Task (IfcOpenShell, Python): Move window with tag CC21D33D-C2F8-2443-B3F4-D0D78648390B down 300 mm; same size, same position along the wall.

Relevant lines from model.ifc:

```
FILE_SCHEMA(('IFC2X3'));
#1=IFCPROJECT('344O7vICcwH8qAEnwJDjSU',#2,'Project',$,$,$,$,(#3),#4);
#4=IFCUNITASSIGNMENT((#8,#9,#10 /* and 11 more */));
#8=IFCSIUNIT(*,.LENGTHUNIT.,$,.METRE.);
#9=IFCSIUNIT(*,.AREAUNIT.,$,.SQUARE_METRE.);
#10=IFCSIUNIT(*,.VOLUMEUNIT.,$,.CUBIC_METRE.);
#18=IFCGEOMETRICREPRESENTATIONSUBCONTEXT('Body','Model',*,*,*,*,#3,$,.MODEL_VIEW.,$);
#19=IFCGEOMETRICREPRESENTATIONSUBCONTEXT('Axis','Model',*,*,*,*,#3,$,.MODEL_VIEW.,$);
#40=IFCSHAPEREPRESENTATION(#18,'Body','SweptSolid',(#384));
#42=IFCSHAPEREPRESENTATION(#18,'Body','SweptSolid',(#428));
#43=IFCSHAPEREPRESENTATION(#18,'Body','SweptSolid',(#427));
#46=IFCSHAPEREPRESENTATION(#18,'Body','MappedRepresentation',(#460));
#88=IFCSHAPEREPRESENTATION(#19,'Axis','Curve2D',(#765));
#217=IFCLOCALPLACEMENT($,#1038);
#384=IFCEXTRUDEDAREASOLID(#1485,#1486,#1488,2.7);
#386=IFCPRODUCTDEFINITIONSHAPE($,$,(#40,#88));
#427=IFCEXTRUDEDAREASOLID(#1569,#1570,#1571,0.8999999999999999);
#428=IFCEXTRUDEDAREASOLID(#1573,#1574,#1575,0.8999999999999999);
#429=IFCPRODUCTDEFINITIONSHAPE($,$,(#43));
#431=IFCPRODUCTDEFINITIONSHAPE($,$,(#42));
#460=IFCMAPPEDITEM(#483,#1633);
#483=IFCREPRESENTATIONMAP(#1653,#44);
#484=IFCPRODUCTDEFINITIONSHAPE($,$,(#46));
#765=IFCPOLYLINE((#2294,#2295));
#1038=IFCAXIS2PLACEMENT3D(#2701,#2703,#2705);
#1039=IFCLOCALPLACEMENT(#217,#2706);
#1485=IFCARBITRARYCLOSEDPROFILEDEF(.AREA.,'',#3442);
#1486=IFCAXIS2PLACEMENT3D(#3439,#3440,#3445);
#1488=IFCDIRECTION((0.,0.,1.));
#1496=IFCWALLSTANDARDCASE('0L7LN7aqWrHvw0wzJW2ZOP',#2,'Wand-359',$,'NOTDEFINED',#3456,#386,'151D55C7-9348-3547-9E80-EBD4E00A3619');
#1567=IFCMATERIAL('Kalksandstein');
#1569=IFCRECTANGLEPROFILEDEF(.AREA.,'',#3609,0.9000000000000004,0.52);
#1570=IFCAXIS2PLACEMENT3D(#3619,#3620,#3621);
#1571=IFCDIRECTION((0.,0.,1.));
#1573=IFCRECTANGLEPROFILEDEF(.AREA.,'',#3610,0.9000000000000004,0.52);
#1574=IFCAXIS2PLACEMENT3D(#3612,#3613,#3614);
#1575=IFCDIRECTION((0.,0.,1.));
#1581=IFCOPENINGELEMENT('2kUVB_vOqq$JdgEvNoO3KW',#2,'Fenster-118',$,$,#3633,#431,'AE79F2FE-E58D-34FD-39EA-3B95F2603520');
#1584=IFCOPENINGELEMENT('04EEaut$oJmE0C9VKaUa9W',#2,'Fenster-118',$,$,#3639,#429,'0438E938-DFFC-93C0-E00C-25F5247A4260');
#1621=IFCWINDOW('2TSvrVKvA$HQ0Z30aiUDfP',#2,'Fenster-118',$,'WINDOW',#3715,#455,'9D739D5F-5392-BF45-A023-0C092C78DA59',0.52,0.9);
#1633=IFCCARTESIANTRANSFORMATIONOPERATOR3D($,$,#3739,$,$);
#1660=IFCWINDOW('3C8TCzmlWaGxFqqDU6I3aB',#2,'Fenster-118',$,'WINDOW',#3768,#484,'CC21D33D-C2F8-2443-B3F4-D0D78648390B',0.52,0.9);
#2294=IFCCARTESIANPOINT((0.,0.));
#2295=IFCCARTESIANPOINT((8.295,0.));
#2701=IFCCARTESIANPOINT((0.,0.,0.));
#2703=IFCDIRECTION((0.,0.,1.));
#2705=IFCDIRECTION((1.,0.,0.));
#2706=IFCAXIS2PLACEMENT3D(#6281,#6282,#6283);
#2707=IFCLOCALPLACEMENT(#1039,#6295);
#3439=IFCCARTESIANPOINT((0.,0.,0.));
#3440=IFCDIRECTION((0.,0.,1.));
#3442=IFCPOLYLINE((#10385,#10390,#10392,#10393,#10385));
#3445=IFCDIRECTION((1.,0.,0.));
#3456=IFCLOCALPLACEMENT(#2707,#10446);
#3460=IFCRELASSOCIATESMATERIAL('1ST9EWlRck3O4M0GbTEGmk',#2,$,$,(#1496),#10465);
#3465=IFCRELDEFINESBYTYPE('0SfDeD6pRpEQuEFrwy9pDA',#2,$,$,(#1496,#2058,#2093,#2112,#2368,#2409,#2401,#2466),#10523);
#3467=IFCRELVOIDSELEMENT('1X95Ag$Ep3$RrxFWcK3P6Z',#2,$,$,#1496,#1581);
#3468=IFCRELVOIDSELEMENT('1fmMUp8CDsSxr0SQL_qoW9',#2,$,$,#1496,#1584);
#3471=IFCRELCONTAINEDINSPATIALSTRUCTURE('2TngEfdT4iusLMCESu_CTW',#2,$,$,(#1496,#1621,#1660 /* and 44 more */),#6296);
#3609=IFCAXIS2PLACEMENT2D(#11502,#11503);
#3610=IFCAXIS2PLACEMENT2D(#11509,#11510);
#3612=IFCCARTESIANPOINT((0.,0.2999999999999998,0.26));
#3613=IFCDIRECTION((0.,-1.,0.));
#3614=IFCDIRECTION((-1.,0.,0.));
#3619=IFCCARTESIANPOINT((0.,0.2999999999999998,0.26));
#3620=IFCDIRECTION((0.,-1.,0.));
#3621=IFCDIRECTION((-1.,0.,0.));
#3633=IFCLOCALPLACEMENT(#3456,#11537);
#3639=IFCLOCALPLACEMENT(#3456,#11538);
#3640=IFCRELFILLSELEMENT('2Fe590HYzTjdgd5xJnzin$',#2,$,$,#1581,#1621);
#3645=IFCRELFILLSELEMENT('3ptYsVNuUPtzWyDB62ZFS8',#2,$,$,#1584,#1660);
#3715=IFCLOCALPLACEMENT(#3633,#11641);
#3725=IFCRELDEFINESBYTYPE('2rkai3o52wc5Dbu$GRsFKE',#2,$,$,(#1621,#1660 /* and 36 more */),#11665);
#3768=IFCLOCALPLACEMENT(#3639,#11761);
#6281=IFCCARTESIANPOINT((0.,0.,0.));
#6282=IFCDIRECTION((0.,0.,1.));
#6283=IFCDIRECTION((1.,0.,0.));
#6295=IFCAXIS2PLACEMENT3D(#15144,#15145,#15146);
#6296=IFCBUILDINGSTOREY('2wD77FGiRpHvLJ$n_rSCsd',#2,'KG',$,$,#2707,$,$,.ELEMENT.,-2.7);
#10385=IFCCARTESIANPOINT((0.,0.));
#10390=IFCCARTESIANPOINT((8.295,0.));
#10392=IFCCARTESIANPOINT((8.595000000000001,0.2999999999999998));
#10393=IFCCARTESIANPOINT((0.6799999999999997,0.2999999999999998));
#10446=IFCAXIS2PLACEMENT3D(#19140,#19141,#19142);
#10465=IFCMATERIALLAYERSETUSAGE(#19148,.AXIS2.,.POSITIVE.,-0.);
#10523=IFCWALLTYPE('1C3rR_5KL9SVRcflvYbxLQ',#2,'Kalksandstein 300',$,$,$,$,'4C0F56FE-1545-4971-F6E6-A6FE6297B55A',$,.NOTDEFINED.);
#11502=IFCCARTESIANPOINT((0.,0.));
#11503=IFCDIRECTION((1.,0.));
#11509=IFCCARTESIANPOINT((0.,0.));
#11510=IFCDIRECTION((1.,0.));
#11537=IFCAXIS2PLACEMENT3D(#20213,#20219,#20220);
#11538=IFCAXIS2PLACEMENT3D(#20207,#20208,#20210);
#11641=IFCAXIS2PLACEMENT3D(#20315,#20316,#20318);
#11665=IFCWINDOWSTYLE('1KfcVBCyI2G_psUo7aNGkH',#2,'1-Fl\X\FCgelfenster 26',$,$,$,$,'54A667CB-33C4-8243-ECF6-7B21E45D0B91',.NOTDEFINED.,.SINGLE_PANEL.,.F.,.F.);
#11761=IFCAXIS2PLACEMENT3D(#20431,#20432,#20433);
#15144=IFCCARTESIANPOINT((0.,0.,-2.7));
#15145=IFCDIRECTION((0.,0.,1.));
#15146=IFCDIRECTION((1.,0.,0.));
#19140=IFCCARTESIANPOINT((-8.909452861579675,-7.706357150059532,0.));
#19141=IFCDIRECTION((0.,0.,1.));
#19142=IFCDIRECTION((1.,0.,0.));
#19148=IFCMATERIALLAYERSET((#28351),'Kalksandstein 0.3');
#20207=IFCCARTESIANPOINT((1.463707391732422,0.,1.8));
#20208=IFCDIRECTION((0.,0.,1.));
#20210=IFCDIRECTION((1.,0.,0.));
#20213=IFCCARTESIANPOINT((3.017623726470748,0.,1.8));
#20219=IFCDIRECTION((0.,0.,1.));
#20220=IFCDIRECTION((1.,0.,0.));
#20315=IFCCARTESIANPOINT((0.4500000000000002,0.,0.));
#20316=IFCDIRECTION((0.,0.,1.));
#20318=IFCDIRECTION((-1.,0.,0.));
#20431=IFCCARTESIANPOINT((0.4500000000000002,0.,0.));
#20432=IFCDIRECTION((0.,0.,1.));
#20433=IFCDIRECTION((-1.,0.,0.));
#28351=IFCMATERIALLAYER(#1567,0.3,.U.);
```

```python
import numpy as np
import ifcopenshell
import ifcopenshell.api.geometry
import ifcopenshell.util.placement
import ifcopenshell.util.unit

model = ifcopenshell.open("model.ifc")
unit_scale = ifcopenshell.util.unit.calculate_unit_scale(model)

window = model.by_id(1660)
opening = window.FillsVoids[0].RelatingOpeningElement
dz = -0.3

shift = np.array([0.0, 0.0, dz])
# The window is placed relative to its opening, so it follows when the opening moves.
matrix = ifcopenshell.util.placement.get_local_placement(opening.ObjectPlacement)
matrix[:3, 3] += shift
ifcopenshell.api.geometry.edit_object_placement(
    model, product=opening, matrix=matrix, is_si=False, should_transform_children=True
)

print(f"moved by {dz * unit_scale:+.3f} m")

model.write("model_v2.ifc")
```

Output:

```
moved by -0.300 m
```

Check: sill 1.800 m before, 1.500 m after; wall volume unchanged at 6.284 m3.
